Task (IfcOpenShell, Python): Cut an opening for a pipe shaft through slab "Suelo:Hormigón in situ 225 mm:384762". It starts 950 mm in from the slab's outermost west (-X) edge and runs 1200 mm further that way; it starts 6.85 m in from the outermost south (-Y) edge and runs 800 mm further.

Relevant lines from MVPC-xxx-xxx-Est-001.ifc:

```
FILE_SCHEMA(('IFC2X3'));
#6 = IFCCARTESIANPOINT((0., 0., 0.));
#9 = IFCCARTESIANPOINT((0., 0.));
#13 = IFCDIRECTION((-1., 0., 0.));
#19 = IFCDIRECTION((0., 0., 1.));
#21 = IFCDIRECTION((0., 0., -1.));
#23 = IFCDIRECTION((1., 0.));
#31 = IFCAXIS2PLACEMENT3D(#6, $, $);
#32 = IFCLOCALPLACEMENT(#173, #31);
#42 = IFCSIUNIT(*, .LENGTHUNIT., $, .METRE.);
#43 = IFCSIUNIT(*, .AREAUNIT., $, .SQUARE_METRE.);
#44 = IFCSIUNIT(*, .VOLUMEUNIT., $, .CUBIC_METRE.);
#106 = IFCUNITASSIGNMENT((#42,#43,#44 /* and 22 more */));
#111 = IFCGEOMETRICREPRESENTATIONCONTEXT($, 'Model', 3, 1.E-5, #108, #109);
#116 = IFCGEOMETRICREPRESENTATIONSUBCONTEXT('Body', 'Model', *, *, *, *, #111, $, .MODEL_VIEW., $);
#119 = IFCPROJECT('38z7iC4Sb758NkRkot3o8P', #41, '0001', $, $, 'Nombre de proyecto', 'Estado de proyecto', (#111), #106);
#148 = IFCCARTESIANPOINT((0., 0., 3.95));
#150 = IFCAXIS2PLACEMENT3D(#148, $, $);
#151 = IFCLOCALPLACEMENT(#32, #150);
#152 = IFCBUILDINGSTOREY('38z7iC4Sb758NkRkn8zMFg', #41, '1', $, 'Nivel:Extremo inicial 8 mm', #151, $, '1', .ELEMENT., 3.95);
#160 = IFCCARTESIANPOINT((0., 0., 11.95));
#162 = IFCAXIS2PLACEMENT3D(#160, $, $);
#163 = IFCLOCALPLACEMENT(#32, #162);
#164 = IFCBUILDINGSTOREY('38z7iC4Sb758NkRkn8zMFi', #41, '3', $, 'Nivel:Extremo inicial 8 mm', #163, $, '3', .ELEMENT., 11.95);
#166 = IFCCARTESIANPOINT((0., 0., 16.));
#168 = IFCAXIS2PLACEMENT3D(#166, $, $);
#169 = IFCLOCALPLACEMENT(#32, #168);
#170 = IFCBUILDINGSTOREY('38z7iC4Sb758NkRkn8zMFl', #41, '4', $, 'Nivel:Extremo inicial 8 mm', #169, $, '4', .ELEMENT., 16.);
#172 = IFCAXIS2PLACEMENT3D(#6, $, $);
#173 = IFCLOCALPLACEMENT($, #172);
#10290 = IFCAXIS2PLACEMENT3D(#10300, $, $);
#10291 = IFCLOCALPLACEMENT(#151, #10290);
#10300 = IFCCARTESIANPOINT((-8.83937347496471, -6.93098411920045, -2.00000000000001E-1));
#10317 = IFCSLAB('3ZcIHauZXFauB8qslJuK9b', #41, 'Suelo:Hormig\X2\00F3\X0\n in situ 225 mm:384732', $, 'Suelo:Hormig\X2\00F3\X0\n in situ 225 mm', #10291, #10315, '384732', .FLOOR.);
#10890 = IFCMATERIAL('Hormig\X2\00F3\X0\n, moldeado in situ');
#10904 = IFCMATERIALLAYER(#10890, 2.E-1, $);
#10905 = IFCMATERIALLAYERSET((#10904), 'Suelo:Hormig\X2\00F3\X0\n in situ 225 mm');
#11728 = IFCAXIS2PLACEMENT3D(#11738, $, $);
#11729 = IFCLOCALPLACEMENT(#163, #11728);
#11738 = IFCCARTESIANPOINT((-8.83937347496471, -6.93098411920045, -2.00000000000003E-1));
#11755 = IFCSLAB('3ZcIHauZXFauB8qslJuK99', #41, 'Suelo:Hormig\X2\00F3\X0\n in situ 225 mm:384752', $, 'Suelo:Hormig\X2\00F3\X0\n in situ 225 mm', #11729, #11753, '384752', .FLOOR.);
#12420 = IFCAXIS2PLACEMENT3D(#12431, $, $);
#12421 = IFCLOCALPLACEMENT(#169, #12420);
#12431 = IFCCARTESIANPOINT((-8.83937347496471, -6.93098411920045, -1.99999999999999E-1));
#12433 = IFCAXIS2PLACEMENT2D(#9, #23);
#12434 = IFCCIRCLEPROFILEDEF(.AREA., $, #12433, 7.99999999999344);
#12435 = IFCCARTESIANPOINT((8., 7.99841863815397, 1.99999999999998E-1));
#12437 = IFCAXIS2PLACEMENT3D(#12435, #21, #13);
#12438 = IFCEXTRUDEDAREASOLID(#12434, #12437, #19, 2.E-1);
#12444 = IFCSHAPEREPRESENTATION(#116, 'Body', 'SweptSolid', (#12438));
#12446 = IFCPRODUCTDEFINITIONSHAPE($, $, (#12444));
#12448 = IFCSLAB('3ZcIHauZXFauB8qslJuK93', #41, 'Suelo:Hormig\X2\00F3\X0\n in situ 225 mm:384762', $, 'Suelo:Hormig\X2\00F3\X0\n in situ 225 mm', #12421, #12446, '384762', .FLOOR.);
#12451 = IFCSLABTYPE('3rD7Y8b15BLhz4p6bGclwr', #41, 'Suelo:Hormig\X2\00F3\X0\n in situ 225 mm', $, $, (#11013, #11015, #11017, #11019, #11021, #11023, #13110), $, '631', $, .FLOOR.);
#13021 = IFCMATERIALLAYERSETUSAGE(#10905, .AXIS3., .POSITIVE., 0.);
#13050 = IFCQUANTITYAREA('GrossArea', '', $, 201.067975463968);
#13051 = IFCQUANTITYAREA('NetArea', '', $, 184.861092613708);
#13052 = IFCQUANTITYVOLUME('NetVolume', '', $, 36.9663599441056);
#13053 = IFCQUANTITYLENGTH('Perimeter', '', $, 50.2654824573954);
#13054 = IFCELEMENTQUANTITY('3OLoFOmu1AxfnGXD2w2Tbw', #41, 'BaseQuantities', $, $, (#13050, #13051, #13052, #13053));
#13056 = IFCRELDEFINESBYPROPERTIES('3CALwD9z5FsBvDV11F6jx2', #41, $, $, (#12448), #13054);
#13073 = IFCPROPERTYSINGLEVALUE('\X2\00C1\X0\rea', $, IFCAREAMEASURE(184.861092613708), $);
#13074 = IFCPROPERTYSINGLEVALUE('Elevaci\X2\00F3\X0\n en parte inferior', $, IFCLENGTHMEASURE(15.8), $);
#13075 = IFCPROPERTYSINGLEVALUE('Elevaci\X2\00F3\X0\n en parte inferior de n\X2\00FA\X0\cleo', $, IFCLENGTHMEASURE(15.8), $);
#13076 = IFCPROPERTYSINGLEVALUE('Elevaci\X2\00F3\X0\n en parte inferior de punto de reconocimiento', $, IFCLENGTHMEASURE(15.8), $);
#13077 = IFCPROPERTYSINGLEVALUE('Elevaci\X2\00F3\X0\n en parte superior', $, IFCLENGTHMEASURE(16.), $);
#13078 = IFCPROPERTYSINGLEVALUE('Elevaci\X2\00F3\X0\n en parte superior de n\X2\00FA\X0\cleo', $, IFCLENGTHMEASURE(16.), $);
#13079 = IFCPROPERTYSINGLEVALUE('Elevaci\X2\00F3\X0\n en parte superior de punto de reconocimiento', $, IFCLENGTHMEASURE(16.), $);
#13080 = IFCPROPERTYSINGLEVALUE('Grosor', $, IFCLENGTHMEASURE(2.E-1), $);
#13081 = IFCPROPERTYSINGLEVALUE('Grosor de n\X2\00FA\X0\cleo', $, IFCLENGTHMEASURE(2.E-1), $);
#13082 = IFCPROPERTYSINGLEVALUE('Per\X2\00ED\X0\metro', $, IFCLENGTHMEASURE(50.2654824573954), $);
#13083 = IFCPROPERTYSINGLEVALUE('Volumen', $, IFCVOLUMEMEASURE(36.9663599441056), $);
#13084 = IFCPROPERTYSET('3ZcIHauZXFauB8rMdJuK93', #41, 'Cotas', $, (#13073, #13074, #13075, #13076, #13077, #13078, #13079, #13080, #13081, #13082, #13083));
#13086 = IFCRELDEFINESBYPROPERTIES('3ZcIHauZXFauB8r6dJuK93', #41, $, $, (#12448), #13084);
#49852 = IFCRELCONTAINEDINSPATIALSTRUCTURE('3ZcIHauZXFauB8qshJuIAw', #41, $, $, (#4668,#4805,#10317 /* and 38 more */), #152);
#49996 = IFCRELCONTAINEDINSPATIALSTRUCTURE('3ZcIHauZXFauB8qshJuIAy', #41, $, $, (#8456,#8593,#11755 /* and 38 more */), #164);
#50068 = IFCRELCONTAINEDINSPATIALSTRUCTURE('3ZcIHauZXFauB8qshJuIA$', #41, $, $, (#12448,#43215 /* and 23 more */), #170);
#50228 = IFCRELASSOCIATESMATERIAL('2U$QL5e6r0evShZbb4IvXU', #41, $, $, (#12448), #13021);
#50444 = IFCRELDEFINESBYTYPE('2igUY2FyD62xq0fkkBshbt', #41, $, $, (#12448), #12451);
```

```python
import numpy as np
import ifcopenshell
import ifcopenshell.api.feature
import ifcopenshell.api.geometry
import ifcopenshell.api.pset
import ifcopenshell.api.root
import ifcopenshell.geom
import ifcopenshell.util.element
import ifcopenshell.util.placement
import ifcopenshell.util.representation
import ifcopenshell.util.shape
import ifcopenshell.util.unit

model = ifcopenshell.open("MVPC-xxx-xxx-Est-001.ifc")
unit_scale = ifcopenshell.util.unit.calculate_unit_scale(model)
area_scale = ifcopenshell.util.unit.calculate_unit_scale(model, "AREAUNIT")
volume_scale = ifcopenshell.util.unit.calculate_unit_scale(model, "VOLUMEUNIT")
settings = ifcopenshell.geom.settings()


def volume(element):
    """Net volume in cubic metres, openings subtracted."""
    shape = ifcopenshell.geom.create_shape(settings, element)
    return ifcopenshell.util.shape.get_volume(shape.geometry)


slab = model.by_guid("3ZcIHauZXFauB8qslJuK93")
before = volume(slab)

# Extent in the slab's own axes, in metres. The edges named are its -X and -Y sides.
slab_shape = ifcopenshell.geom.create_shape(settings, slab)
vertices = ifcopenshell.util.shape.get_vertices(slab_shape.geometry)
x_min, y_min, bottom = vertices.min(axis=0)
top = vertices[:, 2].max()

opening = ifcopenshell.api.root.create_entity(model, ifc_class="IfcOpeningElement", name="Pipe shaft opening")
context = ifcopenshell.util.representation.get_context(model, "Model", "Body", "MODEL_VIEW")
width, depth = 1.2, 0.8
outline = [(0.0, 0.0), (width, 0.0), (width, depth), (0.0, depth), (0.0, 0.0)]
# Overshoot both faces by 50 mm so the cut is clean.
shape = ifcopenshell.api.geometry.add_slab_representation(
    model, context=context, depth=top - bottom + 0.1, polyline=outline
)
ifcopenshell.api.geometry.assign_representation(model, product=opening, representation=shape)

matrix = ifcopenshell.util.placement.get_local_placement(slab.ObjectPlacement)
matrix[:, 3] = matrix @ np.append(np.array([x_min + 0.95, y_min + 6.85, bottom - 0.05]) / unit_scale, 1.0)
ifcopenshell.api.geometry.edit_object_placement(model, product=opening, matrix=matrix, is_si=False)
ifcopenshell.api.feature.add_feature(model, feature=opening, element=slab)

after = volume(slab)

# Update the slab's stored quantities.
qto = model.by_id(ifcopenshell.util.element.get_pset(slab, "BaseQuantities", should_inherit=False)["id"])
ifcopenshell.api.pset.edit_qto(model, qto=qto, properties={
    "NetArea": after / (top - bottom) / area_scale,
    "NetVolume": after / volume_scale,
})
pset = model.by_id(ifcopenshell.util.element.get_pset(slab, "Cotas", should_inherit=False)["id"])
ifcopenshell.api.pset.edit_pset(model, pset=pset, properties={
    "Área": model.create_entity("IfcAreaMeasure", after / (top - bottom) / area_scale),
    "Volumen": model.create_entity("IfcVolumeMeasure", after / volume_scale),
})

print(f"slab volume {before:.3f} -> {after:.3f} m3")

model.write("MVPC-xxx-xxx-Est-001_edited.ifc")
```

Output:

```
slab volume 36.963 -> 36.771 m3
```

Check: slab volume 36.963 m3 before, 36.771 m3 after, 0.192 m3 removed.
